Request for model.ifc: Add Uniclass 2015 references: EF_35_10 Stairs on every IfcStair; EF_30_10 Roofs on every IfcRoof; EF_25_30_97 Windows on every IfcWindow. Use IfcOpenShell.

First a look at what the model holds.

```python
import ifcopenshell

model = ifcopenshell.open("model.ifc")
print(model.schema)
print("classifications:", [c.Name for c in model.by_type("IfcClassification")])
for ifc_class in ("IfcDoor", "IfcRoof", "IfcStair", "IfcWall", "IfcWindow"):
    print(ifc_class, len(model.by_type(ifc_class)))
```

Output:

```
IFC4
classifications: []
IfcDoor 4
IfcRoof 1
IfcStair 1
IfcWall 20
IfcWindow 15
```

```python
import ifcopenshell
import ifcopenshell.api.classification

model = ifcopenshell.open("model.ifc")

system = ifcopenshell.api.classification.add_classification(model, classification="Uniclass 2015")

codes = {
    "IfcStair": ("EF_35_10", "Stairs"),
    "IfcRoof": ("EF_30_10", "Roofs"),
    "IfcWindow": ("EF_25_30_97", "Windows"),
}
for ifc_class, (code, name) in codes.items():
    products = model.by_type(ifc_class)
    ifcopenshell.api.classification.add_reference(
        model, products=products, classification=system, identification=code, name=name
    )
    print(code, len(products))

model.write("model-out.ifc")
```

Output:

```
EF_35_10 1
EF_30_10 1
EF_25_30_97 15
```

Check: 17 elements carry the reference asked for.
